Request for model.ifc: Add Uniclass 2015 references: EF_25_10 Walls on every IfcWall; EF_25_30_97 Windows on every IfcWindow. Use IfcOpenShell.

First a look at what the model holds.

```python
import ifcopenshell

model = ifcopenshell.open("model.ifc")
print(model.schema)
print("classifications:", [c.Name for c in model.by_type("IfcClassification")])
for ifc_class in ("IfcDoor", "IfcRoof", "IfcStair", "IfcWall", "IfcWindow"):
    print(ifc_class, len(model.by_type(ifc_class)))
```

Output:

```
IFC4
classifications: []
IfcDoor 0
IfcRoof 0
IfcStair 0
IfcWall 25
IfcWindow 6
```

```python
import ifcopenshell
import ifcopenshell.api.classification

model = ifcopenshell.open("model.ifc")

system = ifcopenshell.api.classification.add_classification(model, classification="Uniclass 2015")

codes = {
    "IfcWall": ("EF_25_10", "Walls"),
    "IfcWindow": ("EF_25_30_97", "Windows"),
}
for ifc_class, (code, name) in codes.items():
    products = model.by_type(ifc_class)
    ifcopenshell.api.classification.add_reference(
        model, products=products, classification=system, identification=code, name=name
    )
    print(code, len(products))

model.write("model_updated.ifc")
```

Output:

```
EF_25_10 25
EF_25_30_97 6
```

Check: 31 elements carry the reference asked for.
